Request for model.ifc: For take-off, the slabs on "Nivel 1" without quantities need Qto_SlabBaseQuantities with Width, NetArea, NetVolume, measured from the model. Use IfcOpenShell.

First a look at what the model holds.

```python
import ifcopenshell
import ifcopenshell.util.element
import ifcopenshell.util.unit

model = ifcopenshell.open("model.ifc")
print(model.schema)
for unit_type in ("LENGTHUNIT", "AREAUNIT", "VOLUMEUNIT"):
    print(unit_type, ifcopenshell.util.unit.calculate_unit_scale(model, unit_type))
storey = next(s for s in model.by_type("IfcBuildingStorey") if s.Name == "Nivel 1")
slabs = [e for e in ifcopenshell.util.element.get_decomposition(storey) if e.is_a("IfcSlab")]
for e in sorted(slabs, key=lambda e: e.id()):
    print(e.id(), e.is_a(), e.Name, list(ifcopenshell.util.element.get_psets(e, qtos_only=True)), sep=" | ")
```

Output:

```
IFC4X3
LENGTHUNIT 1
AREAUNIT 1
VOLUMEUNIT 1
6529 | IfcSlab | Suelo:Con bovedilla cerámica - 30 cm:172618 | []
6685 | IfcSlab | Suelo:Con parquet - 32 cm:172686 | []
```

```python
import ifcopenshell
import ifcopenshell.api.pset
import ifcopenshell.geom
import ifcopenshell.util.element
import ifcopenshell.util.shape
import ifcopenshell.util.unit

model = ifcopenshell.open("model.ifc")
unit_scale = ifcopenshell.util.unit.calculate_unit_scale(model)
area_scale = ifcopenshell.util.unit.calculate_unit_scale(model, "AREAUNIT")
volume_scale = ifcopenshell.util.unit.calculate_unit_scale(model, "VOLUMEUNIT")
settings = ifcopenshell.geom.settings()

storey = next(s for s in model.by_type("IfcBuildingStorey") if s.Name == "Nivel 1")
slabs = [e for e in ifcopenshell.util.element.get_decomposition(storey) if e.is_a("IfcSlab")]

for e in sorted(slabs, key=lambda e: e.id()):
    if ifcopenshell.util.element.get_psets(e, qtos_only=True, should_inherit=False):
        continue
    # Geometry comes back in metres, in the element's own axes.
    shape = ifcopenshell.geom.create_shape(settings, e)
    values = {
        "Width": ifcopenshell.util.shape.get_z(shape.geometry) / unit_scale,
        "NetArea": ifcopenshell.util.shape.get_footprint_area(shape.geometry) / area_scale,
        "NetVolume": ifcopenshell.util.shape.get_volume(shape.geometry) / volume_scale,
    }
    qto = ifcopenshell.api.pset.add_qto(model, product=e, name="Qto_SlabBaseQuantities")
    ifcopenshell.api.pset.edit_qto(model, qto=qto, properties=values)
    print(e.id(), {k: round(v, 3) for k, v in values.items()})

model.write("model_updated.ifc")
```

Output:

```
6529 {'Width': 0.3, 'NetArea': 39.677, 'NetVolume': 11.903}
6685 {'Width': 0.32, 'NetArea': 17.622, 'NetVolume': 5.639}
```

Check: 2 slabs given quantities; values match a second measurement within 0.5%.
